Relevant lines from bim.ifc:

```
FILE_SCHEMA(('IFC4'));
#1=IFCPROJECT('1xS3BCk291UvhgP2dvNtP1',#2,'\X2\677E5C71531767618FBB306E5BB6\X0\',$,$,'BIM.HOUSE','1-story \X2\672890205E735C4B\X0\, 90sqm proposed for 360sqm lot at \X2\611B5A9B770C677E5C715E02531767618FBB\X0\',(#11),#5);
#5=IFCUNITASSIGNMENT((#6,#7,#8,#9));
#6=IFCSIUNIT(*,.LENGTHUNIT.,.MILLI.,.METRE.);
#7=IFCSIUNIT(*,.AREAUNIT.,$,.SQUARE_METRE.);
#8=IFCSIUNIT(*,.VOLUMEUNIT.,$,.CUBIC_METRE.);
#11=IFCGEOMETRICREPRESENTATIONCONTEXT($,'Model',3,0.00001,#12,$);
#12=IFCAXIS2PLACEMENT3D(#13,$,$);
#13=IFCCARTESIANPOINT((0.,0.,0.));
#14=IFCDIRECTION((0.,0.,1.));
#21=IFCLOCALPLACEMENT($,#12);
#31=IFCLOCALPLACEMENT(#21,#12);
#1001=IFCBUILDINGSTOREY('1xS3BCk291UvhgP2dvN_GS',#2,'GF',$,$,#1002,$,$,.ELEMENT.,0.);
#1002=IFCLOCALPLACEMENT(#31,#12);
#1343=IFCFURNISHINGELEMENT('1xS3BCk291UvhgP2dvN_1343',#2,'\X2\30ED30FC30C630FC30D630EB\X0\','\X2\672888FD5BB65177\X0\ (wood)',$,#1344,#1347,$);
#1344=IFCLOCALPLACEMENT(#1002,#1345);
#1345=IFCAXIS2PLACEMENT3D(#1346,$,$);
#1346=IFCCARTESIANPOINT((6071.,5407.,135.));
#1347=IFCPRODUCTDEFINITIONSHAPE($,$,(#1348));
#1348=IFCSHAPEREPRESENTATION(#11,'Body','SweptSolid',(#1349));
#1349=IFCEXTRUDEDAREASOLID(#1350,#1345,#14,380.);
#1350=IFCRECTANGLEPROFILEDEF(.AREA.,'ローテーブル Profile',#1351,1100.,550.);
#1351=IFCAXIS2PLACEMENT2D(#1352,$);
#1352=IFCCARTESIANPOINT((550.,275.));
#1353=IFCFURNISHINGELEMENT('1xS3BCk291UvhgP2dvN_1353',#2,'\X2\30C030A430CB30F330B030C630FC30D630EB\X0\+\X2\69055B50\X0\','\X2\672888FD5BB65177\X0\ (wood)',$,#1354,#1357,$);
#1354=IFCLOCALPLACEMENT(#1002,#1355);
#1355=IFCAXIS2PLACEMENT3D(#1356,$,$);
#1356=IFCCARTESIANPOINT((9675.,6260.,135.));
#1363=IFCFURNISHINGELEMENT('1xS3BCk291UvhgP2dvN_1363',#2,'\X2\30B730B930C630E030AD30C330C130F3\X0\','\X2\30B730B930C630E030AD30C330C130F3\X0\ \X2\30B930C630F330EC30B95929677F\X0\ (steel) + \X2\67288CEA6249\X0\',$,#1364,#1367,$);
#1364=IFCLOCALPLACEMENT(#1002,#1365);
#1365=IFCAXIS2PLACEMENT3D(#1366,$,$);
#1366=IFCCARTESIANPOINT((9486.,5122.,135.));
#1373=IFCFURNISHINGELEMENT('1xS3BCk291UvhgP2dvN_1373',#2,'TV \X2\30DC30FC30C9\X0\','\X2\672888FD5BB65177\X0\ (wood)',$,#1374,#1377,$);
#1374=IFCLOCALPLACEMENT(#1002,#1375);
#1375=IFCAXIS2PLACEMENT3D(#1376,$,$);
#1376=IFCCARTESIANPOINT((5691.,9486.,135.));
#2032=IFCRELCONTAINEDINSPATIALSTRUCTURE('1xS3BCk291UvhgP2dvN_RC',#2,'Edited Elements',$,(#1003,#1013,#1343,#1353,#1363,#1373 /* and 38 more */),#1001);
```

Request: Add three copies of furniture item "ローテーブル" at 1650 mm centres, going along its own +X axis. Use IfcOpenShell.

```python
import ifcopenshell
import ifcopenshell.api.geometry
import ifcopenshell.api.root
import ifcopenshell.util.element
import ifcopenshell.util.placement
import ifcopenshell.util.unit

model = ifcopenshell.open("bim.ifc")
unit_scale = ifcopenshell.util.unit.calculate_unit_scale(model)


def reuse_history(source, copy):
    """copy_class also copies each property set's owner history, people and application; keep the originals."""
    for rel in copy.IsDefinedBy:
        if rel.is_a("IfcRelDefinesByProperties") and (history := rel.RelatingPropertyDefinition.OwnerHistory):
            rel.RelatingPropertyDefinition.OwnerHistory = source.OwnerHistory
            ifcopenshell.util.element.remove_deep2(model, history)


source = model.by_guid("1xS3BCk291UvhgP2dvN_1343")
base = ifcopenshell.util.placement.get_local_placement(source.ObjectPlacement)
step = base[:3, 0] * 1.65 / unit_scale

for i in range(1, 4):
    copy = ifcopenshell.api.root.copy_class(model, product=source)
    copy.Representation = ifcopenshell.util.element.copy_deep(
        model, source.Representation, exclude=["IfcGeometricRepresentationContext", "IfcRepresentationMap"]
    )
    reuse_history(source, copy)
    matrix = base.copy()
    matrix[:3, 3] += i * step
    print("added at", matrix[:3, 3].round(3) + 0.0)
    ifcopenshell.api.geometry.edit_object_placement(model, product=copy, matrix=matrix, is_si=False)

model.write("bim_edited.ifc")
```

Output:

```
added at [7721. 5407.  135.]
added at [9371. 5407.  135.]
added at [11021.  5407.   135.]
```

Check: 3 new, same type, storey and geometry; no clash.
